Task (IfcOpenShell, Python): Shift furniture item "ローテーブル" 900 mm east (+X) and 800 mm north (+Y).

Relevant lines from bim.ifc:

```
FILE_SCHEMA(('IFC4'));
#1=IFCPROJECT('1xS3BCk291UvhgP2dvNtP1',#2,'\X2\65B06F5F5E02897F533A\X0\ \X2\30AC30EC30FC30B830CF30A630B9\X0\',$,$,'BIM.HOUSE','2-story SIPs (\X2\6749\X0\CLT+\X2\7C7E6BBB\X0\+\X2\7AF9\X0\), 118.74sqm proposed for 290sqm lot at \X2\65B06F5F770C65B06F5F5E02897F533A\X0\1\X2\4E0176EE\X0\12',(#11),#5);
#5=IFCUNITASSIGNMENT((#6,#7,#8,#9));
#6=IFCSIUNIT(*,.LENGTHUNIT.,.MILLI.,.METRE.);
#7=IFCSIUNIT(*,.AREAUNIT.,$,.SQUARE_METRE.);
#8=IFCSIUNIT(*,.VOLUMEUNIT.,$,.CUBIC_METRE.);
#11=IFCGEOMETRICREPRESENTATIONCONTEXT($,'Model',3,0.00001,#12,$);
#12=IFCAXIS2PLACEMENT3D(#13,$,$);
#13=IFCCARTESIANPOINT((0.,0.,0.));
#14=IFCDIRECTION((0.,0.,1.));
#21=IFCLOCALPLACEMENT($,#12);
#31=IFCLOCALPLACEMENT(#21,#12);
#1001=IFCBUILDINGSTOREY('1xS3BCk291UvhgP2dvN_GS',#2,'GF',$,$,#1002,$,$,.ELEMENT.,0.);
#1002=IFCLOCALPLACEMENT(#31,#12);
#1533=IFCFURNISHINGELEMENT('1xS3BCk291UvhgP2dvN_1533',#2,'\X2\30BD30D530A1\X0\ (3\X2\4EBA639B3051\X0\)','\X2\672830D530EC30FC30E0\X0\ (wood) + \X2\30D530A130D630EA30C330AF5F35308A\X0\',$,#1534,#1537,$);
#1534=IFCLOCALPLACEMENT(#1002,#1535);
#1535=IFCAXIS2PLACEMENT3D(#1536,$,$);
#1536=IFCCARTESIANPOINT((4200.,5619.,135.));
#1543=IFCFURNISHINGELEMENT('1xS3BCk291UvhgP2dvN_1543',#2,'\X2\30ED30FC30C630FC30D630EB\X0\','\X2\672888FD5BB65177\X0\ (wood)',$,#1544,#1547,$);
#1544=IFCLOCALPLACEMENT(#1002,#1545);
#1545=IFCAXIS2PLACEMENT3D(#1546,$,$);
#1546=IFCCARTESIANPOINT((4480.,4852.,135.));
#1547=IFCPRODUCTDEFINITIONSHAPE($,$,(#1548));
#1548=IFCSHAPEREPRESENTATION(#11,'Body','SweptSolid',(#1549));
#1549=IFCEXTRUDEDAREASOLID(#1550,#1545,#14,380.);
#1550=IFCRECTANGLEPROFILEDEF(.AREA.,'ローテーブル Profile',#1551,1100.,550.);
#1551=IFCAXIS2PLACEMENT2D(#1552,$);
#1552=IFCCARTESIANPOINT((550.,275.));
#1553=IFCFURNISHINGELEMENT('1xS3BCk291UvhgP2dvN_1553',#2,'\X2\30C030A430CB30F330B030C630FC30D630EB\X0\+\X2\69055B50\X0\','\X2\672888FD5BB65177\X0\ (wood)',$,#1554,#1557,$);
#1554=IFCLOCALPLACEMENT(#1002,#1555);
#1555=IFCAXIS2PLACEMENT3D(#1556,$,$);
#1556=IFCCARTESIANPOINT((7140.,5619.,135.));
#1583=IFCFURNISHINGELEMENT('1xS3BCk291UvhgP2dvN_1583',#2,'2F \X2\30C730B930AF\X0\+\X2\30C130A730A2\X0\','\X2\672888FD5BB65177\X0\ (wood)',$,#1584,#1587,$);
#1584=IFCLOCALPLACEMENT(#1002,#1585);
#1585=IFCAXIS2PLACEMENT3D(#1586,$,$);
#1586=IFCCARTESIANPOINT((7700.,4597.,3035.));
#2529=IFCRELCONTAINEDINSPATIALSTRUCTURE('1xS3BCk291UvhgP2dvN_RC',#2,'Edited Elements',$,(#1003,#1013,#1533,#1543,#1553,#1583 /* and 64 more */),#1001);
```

```python
import ifcopenshell
import ifcopenshell.api.geometry
import ifcopenshell.util.placement

model = ifcopenshell.open("bim.ifc")

item = model.by_guid("1xS3BCk291UvhgP2dvN_1543")
matrix = ifcopenshell.util.placement.get_local_placement(item.ObjectPlacement)
matrix[0, 3] += 900.0
matrix[1, 3] += 800.0
ifcopenshell.api.geometry.edit_object_placement(model, product=item, matrix=matrix, is_si=False)

print(ifcopenshell.util.placement.get_local_placement(item.ObjectPlacement).round(3) + 0.0)

model.write("bim_rev.ifc")
```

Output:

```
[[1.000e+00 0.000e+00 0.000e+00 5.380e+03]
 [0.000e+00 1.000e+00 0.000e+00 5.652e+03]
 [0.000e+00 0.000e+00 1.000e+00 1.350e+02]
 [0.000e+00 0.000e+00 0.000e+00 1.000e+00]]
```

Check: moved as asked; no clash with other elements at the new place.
